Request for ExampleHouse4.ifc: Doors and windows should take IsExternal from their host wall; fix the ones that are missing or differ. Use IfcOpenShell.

First a look at what the model holds.

```python
import ifcopenshell
import ifcopenshell.util.element

model = ifcopenshell.open("ExampleHouse4.ifc")
print(model.schema)
seen = {}
for e in model.by_type("IfcDoor") + model.by_type("IfcWindow"):
    if not e.FillsVoids:
        continue
    host = e.FillsVoids[0].RelatingOpeningElement.VoidsElements[0].RelatingBuildingElement
    own = ifcopenshell.util.element.get_pset(e, f"Pset_{e.is_a()[3:].removesuffix('StandardCase')}Common", "IsExternal")
    wall = ifcopenshell.util.element.get_pset(host, "Pset_WallCommon", "IsExternal")
    seen[e.is_a(), own, wall] = seen.get((e.is_a(), own, wall), 0) + 1
for (cls, own, wall), count in sorted(seen.items(), key=str):
    print(count, cls, "IsExternal:", own, "| host wall:", wall)
```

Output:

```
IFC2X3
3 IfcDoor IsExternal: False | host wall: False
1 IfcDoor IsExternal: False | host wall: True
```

```python
import ifcopenshell
import ifcopenshell.api.pset
import ifcopenshell.util.element

model = ifcopenshell.open("ExampleHouse4.ifc")

count = 0
for ifc_class, pset_name in (("IfcDoor", "Pset_DoorCommon"), ("IfcWindow", "Pset_WindowCommon")):
    for e in model.by_type(ifc_class):
        if not e.FillsVoids:
            continue
        host = e.FillsVoids[0].RelatingOpeningElement.VoidsElements[0].RelatingBuildingElement
        external = ifcopenshell.util.element.get_pset(host, "Pset_WallCommon", "IsExternal")
        if external is None or ifcopenshell.util.element.get_pset(e, pset_name, "IsExternal") == external:
            continue
        pset = ifcopenshell.api.pset.add_pset(model, product=e, name=pset_name)
        ifcopenshell.api.pset.edit_pset(model, pset=pset, properties={"IsExternal": external})
        count += 1

print(count, "updated")

model.write("ExampleHouse4_v2.ifc")
```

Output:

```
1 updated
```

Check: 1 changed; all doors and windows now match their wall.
